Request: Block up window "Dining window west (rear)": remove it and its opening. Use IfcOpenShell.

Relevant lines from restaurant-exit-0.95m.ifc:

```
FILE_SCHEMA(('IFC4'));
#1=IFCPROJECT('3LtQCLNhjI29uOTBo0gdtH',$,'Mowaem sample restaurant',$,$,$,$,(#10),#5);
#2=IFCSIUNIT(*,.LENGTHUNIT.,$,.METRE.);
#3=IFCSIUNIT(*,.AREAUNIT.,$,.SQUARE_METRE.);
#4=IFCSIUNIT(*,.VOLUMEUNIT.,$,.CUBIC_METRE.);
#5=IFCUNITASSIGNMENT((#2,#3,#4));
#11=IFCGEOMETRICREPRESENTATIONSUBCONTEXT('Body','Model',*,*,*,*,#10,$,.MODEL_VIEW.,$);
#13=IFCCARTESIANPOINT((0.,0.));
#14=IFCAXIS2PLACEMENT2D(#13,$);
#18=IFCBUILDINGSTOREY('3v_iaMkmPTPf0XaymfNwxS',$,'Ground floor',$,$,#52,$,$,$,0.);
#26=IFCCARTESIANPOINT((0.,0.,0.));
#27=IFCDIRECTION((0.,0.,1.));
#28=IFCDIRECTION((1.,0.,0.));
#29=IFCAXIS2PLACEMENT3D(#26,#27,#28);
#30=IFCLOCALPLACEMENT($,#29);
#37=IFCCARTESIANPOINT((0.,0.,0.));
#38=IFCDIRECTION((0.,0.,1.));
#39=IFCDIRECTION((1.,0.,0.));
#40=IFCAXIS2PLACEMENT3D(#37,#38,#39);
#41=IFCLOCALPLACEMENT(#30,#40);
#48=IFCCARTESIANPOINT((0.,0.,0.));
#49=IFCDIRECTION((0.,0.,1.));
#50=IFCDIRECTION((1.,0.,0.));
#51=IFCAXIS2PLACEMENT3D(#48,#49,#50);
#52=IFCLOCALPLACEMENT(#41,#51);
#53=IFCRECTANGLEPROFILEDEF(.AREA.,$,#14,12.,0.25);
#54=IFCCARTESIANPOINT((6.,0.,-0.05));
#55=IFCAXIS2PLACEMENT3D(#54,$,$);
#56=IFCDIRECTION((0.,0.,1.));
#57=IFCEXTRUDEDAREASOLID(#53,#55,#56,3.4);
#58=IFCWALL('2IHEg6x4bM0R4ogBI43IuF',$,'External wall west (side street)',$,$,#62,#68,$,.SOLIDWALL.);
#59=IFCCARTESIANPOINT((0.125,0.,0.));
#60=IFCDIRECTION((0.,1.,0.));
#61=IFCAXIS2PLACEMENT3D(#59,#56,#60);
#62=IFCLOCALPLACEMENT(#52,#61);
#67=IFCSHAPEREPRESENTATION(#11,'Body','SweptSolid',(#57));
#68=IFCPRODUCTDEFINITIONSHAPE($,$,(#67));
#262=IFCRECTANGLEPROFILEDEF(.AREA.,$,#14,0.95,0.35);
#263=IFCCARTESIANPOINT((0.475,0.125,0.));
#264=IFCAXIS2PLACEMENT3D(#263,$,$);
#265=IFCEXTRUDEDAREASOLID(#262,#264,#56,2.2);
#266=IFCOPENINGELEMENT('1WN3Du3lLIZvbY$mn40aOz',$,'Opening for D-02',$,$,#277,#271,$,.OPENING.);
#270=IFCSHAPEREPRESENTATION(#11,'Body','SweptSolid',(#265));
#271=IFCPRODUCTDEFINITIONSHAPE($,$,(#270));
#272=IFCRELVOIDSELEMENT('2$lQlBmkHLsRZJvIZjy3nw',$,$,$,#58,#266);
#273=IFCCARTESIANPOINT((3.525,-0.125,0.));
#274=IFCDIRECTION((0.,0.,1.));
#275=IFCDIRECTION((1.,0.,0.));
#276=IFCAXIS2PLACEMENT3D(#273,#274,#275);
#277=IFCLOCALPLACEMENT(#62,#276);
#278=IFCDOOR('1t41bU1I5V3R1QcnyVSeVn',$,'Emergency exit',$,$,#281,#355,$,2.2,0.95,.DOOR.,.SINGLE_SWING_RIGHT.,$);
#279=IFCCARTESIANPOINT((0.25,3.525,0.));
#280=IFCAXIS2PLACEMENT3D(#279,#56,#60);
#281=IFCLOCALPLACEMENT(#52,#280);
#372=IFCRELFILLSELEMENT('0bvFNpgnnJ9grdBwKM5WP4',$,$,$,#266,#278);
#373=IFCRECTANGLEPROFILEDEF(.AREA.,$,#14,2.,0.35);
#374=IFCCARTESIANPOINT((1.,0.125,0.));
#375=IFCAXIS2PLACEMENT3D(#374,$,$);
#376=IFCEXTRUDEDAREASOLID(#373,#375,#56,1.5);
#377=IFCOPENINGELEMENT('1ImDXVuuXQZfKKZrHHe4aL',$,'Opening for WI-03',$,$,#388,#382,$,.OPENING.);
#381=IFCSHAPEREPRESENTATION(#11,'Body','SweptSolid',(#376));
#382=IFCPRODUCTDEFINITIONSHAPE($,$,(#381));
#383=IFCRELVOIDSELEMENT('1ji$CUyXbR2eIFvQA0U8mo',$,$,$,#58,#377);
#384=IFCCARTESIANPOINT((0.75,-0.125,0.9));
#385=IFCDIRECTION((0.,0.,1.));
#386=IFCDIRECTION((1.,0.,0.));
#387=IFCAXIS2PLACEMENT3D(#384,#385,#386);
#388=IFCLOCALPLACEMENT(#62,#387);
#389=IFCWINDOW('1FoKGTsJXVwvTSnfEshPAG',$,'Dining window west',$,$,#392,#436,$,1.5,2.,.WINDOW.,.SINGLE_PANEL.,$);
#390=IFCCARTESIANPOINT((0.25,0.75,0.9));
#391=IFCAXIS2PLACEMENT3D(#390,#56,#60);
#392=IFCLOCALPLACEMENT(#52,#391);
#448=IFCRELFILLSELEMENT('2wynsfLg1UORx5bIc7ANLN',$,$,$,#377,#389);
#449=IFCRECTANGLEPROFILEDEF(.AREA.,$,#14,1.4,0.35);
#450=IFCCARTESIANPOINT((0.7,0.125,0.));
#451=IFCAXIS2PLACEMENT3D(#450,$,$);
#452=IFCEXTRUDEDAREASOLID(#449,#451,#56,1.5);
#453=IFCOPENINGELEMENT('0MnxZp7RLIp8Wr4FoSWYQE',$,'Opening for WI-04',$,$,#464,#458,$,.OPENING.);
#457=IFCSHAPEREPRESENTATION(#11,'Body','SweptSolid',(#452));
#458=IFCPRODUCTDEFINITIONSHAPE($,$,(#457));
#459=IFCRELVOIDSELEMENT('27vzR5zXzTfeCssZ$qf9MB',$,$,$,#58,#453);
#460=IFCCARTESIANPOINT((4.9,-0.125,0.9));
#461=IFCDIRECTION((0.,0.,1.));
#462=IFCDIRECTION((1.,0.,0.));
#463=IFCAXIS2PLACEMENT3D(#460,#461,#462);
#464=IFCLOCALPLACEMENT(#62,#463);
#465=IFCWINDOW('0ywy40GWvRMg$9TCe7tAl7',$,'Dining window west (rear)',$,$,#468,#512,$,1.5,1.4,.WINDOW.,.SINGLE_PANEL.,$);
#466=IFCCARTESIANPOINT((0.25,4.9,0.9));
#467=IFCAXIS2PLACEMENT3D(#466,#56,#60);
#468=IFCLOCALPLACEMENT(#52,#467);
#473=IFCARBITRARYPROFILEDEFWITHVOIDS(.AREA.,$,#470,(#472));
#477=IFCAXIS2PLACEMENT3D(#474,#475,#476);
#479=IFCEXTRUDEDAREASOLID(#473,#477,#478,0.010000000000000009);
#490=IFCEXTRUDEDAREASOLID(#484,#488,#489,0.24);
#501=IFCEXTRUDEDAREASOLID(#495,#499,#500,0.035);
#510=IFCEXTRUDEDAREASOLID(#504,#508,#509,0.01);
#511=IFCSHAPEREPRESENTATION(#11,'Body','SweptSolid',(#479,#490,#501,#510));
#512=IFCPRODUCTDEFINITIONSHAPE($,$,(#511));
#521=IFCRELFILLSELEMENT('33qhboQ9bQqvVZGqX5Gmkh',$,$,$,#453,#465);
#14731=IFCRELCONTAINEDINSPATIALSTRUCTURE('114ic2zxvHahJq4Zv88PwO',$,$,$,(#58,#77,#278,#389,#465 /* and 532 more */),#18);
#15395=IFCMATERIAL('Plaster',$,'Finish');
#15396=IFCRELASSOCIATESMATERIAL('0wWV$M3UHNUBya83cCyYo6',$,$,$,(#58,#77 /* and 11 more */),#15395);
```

```python
import ifcopenshell
import ifcopenshell.api.feature
import ifcopenshell.api.root
import ifcopenshell.geom
import ifcopenshell.util.shape

model = ifcopenshell.open("restaurant-exit-0.95m.ifc")
settings = ifcopenshell.geom.settings()


def volume(element):
    """Net volume in cubic metres, openings subtracted."""
    shape = ifcopenshell.geom.create_shape(settings, element)
    return ifcopenshell.util.shape.get_volume(shape.geometry)


window = model.by_guid("0ywy40GWvRMg$9TCe7tAl7")
opening = window.FillsVoids[0].RelatingOpeningElement
wall = opening.VoidsElements[0].RelatingBuildingElement
before = volume(wall)

ifcopenshell.api.root.remove_product(model, product=window)
ifcopenshell.api.feature.remove_feature(model, feature=opening)

after = volume(wall)

print(f"wall volume {before:.3f} -> {after:.3f} m3")

model.write("restaurant-exit-0.95m-out.ifc")
```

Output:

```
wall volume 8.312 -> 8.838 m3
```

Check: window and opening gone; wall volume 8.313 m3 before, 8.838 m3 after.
